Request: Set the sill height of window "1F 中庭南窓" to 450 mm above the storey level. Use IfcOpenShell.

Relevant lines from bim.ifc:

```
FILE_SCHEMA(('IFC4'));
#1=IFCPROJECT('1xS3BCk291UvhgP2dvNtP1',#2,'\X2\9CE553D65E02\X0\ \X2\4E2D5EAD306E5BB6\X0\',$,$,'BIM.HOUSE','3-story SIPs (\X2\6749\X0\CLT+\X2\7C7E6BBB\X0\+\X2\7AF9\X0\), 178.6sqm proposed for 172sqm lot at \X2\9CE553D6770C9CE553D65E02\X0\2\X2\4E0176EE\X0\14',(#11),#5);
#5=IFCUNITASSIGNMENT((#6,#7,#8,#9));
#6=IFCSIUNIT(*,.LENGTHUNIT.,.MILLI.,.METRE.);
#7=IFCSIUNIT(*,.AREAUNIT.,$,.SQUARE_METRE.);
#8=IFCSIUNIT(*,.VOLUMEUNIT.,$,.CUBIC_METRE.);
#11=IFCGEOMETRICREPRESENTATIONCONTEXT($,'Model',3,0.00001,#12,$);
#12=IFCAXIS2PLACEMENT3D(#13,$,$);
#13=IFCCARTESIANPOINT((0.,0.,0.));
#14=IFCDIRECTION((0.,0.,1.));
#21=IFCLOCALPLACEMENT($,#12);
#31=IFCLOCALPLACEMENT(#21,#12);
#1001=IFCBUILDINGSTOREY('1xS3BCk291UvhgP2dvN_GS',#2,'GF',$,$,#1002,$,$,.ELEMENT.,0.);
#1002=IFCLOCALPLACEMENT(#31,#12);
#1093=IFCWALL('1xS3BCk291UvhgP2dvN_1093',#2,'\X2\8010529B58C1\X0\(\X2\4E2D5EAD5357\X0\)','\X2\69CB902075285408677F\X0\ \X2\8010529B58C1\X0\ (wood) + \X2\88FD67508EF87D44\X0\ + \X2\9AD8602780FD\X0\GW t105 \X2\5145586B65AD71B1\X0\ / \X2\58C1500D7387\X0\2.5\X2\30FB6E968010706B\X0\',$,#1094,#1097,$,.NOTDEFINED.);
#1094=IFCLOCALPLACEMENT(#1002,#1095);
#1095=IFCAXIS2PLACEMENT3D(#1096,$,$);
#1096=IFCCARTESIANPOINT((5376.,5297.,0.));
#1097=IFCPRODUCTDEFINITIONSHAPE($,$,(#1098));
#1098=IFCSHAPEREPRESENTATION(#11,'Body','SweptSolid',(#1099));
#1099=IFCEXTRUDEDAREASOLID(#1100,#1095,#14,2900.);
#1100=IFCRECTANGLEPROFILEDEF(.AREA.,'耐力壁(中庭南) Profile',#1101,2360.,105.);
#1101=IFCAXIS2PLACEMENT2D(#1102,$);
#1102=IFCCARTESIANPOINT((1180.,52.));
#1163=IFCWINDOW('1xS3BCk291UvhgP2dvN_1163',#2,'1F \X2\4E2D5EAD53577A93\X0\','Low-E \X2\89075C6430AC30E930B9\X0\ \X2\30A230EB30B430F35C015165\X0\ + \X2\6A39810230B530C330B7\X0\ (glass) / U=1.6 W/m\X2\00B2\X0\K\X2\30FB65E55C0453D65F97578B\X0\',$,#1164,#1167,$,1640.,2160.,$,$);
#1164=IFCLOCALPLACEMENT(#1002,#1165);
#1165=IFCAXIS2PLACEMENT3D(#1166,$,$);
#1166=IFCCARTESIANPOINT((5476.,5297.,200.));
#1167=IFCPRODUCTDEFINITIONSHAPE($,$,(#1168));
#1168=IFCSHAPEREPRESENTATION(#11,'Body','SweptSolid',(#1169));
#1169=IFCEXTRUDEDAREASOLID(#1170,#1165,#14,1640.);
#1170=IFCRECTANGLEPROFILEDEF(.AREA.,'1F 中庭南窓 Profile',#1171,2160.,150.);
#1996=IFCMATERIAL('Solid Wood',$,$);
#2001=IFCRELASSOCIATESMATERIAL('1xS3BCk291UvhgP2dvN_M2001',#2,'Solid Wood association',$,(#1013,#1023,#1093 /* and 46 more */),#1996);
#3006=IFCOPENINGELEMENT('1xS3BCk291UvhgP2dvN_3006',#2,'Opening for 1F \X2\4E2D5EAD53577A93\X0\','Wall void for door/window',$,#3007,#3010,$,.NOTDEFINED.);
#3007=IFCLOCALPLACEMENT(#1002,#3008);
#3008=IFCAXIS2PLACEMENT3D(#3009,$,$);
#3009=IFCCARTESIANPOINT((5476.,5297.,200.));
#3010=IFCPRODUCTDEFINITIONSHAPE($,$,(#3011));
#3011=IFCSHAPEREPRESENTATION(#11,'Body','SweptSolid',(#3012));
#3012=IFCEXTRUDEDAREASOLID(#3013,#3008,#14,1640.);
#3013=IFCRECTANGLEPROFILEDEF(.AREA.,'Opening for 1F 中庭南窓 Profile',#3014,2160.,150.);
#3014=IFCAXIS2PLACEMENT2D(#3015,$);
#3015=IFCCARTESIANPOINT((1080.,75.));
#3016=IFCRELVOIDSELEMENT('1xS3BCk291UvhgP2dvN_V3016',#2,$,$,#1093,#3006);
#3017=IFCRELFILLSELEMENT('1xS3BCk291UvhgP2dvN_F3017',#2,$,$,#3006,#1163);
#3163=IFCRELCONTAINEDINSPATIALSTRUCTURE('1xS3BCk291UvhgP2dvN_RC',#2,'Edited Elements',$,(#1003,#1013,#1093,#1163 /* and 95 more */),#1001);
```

```python
import numpy as np
import ifcopenshell
import ifcopenshell.api.geometry
import ifcopenshell.geom
import ifcopenshell.util.element
import ifcopenshell.util.placement
import ifcopenshell.util.shape
import ifcopenshell.util.unit

model = ifcopenshell.open("bim.ifc")
unit_scale = ifcopenshell.util.unit.calculate_unit_scale(model)

window = model.by_guid("1xS3BCk291UvhgP2dvN_1163")
opening = window.FillsVoids[0].RelatingOpeningElement
storey = ifcopenshell.util.element.get_container(window, ifc_class="IfcBuildingStorey")
level = ifcopenshell.util.placement.get_local_placement(storey.ObjectPlacement)[2, 3]

# The opening's origin need not be at the sill, so measure its lowest point.
shape = ifcopenshell.geom.create_shape(ifcopenshell.geom.settings(), opening)
bottom = ifcopenshell.util.shape.get_shape_bottom_elevation(shape, shape.geometry) / unit_scale
dz = level + 450.0 - bottom

shift = np.array([0.0, 0.0, dz])
# The window is not placed relative to its opening, so move both.
for product in (opening, window):
    matrix = ifcopenshell.util.placement.get_local_placement(product.ObjectPlacement)
    matrix[:3, 3] += shift
    ifcopenshell.api.geometry.edit_object_placement(model, product=product, matrix=matrix, is_si=False)

print(f"moved by {dz * unit_scale:+.3f} m")

model.write("bim_updated.ifc")
```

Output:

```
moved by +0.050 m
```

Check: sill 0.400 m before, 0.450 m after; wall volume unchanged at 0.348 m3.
